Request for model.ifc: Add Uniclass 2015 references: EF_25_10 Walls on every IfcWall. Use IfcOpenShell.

First a look at what the model holds.

```python
import ifcopenshell

model = ifcopenshell.open("model.ifc")
print(model.schema)
print("classifications:", [c.Name for c in model.by_type("IfcClassification")])
for ifc_class in ("IfcDoor", "IfcRoof", "IfcStair", "IfcWall", "IfcWindow"):
    print(ifc_class, len(model.by_type(ifc_class)))
```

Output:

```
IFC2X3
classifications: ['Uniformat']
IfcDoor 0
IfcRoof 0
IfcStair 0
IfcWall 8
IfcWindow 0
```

```python
import ifcopenshell
import ifcopenshell.api.classification

model = ifcopenshell.open("model.ifc")

# IFC2X3 requires Source and Edition and has no link from the project to the system.
system = model.create_entity("IfcClassification", Source="NBS", Edition="2015", Name="Uniclass 2015")

codes = {
    "IfcWall": ("EF_25_10", "Walls"),
}
for ifc_class, (code, name) in codes.items():
    products = model.by_type(ifc_class)
    ifcopenshell.api.classification.add_reference(
        model, products=products, classification=system, identification=code, name=name
    )
    print(code, len(products))

model.write("model_updated.ifc")
```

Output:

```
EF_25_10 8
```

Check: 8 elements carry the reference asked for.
